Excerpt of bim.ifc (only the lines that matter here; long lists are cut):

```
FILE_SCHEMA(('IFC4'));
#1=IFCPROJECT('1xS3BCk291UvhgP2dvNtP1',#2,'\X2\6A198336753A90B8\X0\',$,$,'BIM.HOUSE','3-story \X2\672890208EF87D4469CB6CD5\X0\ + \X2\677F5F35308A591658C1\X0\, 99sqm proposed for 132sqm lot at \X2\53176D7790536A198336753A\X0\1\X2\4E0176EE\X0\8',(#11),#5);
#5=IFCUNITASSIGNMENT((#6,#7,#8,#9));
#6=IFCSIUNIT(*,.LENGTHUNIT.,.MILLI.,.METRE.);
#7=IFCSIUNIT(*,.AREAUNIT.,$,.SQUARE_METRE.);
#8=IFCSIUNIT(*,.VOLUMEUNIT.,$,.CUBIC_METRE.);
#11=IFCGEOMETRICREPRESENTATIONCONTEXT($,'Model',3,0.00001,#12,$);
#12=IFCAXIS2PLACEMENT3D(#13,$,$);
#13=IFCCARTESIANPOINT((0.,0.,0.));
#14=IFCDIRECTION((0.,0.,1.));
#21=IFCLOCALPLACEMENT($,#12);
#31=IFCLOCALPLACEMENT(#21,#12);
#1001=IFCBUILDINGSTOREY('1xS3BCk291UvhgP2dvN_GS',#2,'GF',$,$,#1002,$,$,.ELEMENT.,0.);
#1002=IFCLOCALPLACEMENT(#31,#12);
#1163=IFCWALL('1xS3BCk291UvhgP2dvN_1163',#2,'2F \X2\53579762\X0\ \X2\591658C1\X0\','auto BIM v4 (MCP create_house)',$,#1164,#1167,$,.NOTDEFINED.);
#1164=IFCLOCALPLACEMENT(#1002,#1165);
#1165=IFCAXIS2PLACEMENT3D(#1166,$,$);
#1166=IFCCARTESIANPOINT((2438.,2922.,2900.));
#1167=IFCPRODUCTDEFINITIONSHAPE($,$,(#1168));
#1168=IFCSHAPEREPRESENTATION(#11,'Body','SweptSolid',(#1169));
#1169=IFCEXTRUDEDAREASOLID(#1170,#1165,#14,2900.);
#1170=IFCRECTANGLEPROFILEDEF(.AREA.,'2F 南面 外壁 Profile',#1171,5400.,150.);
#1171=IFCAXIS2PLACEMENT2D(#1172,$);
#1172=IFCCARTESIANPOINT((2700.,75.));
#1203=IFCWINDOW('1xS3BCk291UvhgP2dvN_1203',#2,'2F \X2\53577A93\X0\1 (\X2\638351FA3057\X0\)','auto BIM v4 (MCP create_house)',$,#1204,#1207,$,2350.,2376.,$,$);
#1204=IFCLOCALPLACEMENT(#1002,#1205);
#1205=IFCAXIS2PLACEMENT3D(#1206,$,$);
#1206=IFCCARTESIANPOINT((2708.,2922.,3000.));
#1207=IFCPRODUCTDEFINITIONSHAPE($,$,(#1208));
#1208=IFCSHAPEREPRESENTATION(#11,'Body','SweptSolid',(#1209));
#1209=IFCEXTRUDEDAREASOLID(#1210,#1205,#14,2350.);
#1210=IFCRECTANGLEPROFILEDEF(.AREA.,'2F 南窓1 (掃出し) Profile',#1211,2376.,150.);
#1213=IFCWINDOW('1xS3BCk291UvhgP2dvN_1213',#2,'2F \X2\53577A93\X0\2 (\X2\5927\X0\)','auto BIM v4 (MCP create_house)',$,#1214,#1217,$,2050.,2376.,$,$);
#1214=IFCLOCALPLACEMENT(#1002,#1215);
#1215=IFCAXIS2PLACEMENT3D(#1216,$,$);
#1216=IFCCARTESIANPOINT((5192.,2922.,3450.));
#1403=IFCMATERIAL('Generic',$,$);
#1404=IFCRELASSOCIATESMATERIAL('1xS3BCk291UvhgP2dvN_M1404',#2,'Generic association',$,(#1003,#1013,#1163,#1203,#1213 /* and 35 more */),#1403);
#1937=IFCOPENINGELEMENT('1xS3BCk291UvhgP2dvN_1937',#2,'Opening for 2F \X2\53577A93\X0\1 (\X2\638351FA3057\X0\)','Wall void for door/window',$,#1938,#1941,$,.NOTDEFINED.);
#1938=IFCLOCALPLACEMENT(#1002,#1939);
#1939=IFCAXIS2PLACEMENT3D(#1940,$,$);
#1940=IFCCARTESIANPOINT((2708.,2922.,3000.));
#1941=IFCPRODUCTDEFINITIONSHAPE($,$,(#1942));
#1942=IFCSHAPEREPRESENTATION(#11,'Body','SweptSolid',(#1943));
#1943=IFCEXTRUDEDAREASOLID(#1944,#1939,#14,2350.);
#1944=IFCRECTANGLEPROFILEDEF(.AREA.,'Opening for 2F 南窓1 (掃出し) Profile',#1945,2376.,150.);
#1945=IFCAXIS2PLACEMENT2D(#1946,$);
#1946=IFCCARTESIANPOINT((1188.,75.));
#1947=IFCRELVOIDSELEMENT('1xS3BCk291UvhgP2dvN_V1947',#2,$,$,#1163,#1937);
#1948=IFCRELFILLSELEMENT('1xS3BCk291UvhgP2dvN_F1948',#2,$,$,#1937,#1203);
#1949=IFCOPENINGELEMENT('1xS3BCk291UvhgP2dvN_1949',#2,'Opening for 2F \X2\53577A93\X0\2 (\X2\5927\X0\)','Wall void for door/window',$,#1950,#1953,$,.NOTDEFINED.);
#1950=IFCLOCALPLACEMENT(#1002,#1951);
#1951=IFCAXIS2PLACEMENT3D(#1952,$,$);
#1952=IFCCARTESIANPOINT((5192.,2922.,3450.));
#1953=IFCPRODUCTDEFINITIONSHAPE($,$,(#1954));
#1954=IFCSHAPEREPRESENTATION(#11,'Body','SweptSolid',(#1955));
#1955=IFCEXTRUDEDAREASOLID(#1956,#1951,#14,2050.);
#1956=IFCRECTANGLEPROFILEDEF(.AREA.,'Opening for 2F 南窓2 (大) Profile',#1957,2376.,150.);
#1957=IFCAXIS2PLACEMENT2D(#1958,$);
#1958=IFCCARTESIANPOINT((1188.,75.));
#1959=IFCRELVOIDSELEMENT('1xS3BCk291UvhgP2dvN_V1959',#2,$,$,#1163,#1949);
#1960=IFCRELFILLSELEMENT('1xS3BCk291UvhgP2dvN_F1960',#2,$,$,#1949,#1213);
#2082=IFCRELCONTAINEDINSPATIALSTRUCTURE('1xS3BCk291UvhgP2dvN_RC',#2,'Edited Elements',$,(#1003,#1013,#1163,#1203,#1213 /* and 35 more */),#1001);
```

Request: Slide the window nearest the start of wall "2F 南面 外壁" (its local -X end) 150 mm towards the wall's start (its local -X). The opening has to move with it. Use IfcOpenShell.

```python
import ifcopenshell
import ifcopenshell.api.geometry
import ifcopenshell.util.placement
import ifcopenshell.util.unit

model = ifcopenshell.open("bim.ifc")
unit_scale = ifcopenshell.util.unit.calculate_unit_scale(model)

window = model.by_id(1203)
opening = window.FillsVoids[0].RelatingOpeningElement
wall = opening.VoidsElements[0].RelatingBuildingElement

wall_matrix = ifcopenshell.util.placement.get_local_placement(wall.ObjectPlacement)
shift = wall_matrix[:3, 0] * -0.15 / unit_scale
before = ifcopenshell.util.placement.get_local_placement(window.ObjectPlacement)[:3, 3].copy()

# The window is not placed relative to its opening, so move both.
for product in (opening, window):
    matrix = ifcopenshell.util.placement.get_local_placement(product.ObjectPlacement)
    matrix[:3, 3] += shift
    ifcopenshell.api.geometry.edit_object_placement(model, product=product, matrix=matrix, is_si=False)

after = ifcopenshell.util.placement.get_local_placement(window.ObjectPlacement)[:3, 3]
print("window moved by", (after - before).round(3) + 0.0)

model.write("bim_edited.ifc")
```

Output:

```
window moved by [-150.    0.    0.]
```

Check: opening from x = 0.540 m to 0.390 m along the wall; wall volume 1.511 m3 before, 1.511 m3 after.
